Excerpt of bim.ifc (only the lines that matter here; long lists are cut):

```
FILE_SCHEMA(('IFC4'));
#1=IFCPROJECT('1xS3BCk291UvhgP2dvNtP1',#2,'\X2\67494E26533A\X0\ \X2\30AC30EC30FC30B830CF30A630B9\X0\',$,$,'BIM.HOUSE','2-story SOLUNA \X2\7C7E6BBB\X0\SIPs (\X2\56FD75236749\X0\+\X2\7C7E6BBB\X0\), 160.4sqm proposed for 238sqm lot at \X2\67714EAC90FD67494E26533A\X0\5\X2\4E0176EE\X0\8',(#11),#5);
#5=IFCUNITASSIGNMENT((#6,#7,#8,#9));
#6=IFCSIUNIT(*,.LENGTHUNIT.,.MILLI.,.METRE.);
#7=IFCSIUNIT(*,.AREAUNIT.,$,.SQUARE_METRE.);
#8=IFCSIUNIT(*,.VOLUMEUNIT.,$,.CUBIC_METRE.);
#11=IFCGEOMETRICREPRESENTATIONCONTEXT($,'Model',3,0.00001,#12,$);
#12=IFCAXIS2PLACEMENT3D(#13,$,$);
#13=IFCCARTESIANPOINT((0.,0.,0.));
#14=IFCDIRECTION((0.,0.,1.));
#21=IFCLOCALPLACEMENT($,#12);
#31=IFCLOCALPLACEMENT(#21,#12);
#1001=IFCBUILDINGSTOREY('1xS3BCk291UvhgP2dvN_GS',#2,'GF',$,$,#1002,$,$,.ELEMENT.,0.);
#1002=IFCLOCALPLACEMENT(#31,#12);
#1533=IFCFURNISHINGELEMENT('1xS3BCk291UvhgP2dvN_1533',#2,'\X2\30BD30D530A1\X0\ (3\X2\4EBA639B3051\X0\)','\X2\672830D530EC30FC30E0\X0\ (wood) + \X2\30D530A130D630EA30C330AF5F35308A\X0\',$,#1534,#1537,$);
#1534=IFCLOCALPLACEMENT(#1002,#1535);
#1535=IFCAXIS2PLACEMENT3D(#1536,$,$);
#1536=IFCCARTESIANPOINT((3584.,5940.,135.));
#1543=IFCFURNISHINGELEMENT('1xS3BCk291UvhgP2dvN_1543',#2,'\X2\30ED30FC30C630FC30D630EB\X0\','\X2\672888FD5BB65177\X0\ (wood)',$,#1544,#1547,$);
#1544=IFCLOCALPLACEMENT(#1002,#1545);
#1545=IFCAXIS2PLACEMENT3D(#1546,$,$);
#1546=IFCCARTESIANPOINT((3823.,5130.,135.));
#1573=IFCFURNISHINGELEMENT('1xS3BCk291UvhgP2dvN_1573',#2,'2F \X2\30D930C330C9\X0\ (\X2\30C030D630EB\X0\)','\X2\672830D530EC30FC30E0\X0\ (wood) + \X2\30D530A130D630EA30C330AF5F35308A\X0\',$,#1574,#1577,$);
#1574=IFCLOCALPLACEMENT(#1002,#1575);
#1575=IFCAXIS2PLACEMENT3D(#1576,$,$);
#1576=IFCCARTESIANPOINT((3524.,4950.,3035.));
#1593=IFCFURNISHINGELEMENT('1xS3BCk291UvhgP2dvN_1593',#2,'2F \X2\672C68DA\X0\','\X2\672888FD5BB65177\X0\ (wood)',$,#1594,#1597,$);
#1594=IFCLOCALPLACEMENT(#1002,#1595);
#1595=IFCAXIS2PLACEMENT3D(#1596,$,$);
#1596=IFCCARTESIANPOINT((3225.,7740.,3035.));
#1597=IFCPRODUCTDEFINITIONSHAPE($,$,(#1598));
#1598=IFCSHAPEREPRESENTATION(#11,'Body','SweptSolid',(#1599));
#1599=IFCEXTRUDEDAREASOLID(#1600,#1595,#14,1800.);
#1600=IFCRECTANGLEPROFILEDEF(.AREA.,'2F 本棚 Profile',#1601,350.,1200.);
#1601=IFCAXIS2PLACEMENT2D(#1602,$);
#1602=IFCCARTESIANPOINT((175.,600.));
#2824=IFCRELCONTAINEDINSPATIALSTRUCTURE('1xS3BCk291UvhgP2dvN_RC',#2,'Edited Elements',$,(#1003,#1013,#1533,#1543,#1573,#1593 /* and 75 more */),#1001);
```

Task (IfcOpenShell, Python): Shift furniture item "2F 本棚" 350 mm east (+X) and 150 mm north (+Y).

```python
import ifcopenshell
import ifcopenshell.api.geometry
import ifcopenshell.util.placement

model = ifcopenshell.open("bim.ifc")

item = model.by_guid("1xS3BCk291UvhgP2dvN_1593")
matrix = ifcopenshell.util.placement.get_local_placement(item.ObjectPlacement)
matrix[0, 3] += 350.0
matrix[1, 3] += 150.0
ifcopenshell.api.geometry.edit_object_placement(model, product=item, matrix=matrix, is_si=False)

print(ifcopenshell.util.placement.get_local_placement(item.ObjectPlacement).round(3) + 0.0)

model.write("bim_rev.ifc")
```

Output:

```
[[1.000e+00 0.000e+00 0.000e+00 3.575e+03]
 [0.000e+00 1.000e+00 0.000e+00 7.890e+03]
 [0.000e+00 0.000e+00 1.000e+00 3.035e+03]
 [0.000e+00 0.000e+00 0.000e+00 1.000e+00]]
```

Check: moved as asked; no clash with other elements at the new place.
